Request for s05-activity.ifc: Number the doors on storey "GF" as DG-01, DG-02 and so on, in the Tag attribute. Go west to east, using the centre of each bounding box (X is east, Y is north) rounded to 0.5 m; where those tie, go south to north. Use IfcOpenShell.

First a look at what the model holds.

```python
import ifcopenshell
import ifcopenshell.util.element
import ifcopenshell.util.placement

model = ifcopenshell.open("s05-activity.ifc")
print(model.schema)
storey = next(s for s in model.by_type("IfcBuildingStorey") if s.Name == "GF")
doors = [e for e in ifcopenshell.util.element.get_decomposition(storey) if e.is_a("IfcDoor")]
for e in sorted(doors, key=lambda e: e.id()):
    origin = ifcopenshell.util.placement.get_local_placement(e.ObjectPlacement)[:3, 3]
    print(e.id(), e.Tag, e.Name, origin.round(2) + 0.0, sep=" | ")
```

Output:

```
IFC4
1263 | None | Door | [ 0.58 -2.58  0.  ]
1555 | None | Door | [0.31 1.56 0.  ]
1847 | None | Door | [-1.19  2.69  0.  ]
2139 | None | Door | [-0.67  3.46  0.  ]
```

```python
import ifcopenshell
import ifcopenshell.geom
import ifcopenshell.util.element
import ifcopenshell.util.shape

model = ifcopenshell.open("s05-activity.ifc")
settings = ifcopenshell.geom.settings()
settings.set("use-world-coords", True)


def centre(element):
    shape = ifcopenshell.geom.create_shape(settings, element)
    return ifcopenshell.util.shape.get_bbox_centroid(shape.geometry)


storey = next(s for s in model.by_type("IfcBuildingStorey") if s.Name == "GF")
doors = [e for e in ifcopenshell.util.element.get_decomposition(storey) if e.is_a("IfcDoor")]

# Insertion points can sit at a corner or the storey origin, so sort by the geometry (in metres).
centres = {e: centre(e) for e in doors}
doors.sort(key=lambda e: (round(centres[e][0] / 0.5), centres[e][1]))

for i, e in enumerate(doors, start=1):
    number = f"DG-{i:02d}"
    e.Tag = number
    print(e.id(), number)

model.write("s05-activity_v2.ifc")
```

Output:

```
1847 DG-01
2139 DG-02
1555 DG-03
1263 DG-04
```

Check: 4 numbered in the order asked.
